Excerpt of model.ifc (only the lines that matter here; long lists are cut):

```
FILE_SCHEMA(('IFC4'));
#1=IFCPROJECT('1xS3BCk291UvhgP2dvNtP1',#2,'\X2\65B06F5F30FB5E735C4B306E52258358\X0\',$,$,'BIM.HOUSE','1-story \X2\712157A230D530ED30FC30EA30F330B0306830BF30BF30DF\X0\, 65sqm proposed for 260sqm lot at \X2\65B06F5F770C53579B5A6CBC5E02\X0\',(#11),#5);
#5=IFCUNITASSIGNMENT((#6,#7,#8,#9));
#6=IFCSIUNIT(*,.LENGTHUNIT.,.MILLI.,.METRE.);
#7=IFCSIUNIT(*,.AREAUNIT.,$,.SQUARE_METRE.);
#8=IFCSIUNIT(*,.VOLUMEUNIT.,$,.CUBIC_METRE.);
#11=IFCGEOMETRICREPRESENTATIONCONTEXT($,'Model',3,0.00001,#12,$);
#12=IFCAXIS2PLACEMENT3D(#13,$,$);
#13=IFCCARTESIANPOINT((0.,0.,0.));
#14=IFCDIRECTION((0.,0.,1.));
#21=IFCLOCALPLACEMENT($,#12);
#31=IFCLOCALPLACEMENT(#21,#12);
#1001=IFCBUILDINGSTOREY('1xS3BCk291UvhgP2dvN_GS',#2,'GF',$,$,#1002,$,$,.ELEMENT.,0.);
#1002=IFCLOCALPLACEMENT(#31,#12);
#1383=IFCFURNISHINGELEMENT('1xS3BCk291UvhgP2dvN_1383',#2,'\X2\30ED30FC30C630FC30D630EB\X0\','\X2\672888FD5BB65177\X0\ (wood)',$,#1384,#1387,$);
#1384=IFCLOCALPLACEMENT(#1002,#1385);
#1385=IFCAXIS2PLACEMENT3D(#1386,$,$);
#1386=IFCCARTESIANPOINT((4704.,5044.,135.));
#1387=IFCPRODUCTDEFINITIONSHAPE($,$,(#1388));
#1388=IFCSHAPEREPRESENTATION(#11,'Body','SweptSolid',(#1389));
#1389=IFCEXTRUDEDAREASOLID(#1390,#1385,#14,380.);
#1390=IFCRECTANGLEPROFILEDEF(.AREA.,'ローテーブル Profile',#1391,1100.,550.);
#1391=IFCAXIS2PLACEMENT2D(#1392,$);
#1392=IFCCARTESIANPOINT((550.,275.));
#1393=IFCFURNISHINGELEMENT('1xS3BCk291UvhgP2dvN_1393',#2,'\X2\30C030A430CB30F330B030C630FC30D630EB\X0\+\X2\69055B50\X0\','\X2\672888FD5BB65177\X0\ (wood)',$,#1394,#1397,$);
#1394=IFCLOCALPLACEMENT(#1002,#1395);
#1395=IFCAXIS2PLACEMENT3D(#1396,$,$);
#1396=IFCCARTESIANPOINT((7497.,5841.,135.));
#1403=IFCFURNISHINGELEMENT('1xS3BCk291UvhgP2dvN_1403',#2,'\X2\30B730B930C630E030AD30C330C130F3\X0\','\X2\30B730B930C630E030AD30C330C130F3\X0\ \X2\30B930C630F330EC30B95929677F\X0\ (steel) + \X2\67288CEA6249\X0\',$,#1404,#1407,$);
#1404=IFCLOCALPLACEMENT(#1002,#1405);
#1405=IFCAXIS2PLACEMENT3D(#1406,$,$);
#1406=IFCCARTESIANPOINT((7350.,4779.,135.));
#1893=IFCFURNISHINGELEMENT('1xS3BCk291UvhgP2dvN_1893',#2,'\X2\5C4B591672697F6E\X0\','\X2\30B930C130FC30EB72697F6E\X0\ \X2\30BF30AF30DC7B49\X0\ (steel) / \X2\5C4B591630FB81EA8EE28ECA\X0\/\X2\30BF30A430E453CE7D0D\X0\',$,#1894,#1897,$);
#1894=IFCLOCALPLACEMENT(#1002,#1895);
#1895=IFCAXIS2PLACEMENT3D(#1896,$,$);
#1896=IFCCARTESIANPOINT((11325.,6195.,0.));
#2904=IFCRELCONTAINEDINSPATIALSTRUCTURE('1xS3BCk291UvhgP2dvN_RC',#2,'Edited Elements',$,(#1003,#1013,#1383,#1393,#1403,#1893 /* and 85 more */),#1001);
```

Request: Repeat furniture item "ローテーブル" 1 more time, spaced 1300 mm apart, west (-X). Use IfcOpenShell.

```python
import numpy as np
import ifcopenshell
import ifcopenshell.api.geometry
import ifcopenshell.api.root
import ifcopenshell.util.element
import ifcopenshell.util.placement
import ifcopenshell.util.unit

model = ifcopenshell.open("model.ifc")
unit_scale = ifcopenshell.util.unit.calculate_unit_scale(model)


def reuse_history(source, copy):
    """copy_class also copies each property set's owner history, people and application; keep the originals."""
    for rel in copy.IsDefinedBy:
        if rel.is_a("IfcRelDefinesByProperties") and (history := rel.RelatingPropertyDefinition.OwnerHistory):
            rel.RelatingPropertyDefinition.OwnerHistory = source.OwnerHistory
            ifcopenshell.util.element.remove_deep2(model, history)


source = model.by_guid("1xS3BCk291UvhgP2dvN_1383")
base = ifcopenshell.util.placement.get_local_placement(source.ObjectPlacement)
step = np.array([-1.0, 0.0, 0.0]) * 1.3 / unit_scale

for i in range(1, 2):
    copy = ifcopenshell.api.root.copy_class(model, product=source)
    copy.Representation = ifcopenshell.util.element.copy_deep(
        model, source.Representation, exclude=["IfcGeometricRepresentationContext", "IfcRepresentationMap"]
    )
    reuse_history(source, copy)
    matrix = base.copy()
    matrix[:3, 3] += i * step
    print("added at", matrix[:3, 3].round(3) + 0.0)
    ifcopenshell.api.geometry.edit_object_placement(model, product=copy, matrix=matrix, is_si=False)

model.write("model_rev.ifc")
```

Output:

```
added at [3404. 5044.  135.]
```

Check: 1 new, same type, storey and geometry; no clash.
